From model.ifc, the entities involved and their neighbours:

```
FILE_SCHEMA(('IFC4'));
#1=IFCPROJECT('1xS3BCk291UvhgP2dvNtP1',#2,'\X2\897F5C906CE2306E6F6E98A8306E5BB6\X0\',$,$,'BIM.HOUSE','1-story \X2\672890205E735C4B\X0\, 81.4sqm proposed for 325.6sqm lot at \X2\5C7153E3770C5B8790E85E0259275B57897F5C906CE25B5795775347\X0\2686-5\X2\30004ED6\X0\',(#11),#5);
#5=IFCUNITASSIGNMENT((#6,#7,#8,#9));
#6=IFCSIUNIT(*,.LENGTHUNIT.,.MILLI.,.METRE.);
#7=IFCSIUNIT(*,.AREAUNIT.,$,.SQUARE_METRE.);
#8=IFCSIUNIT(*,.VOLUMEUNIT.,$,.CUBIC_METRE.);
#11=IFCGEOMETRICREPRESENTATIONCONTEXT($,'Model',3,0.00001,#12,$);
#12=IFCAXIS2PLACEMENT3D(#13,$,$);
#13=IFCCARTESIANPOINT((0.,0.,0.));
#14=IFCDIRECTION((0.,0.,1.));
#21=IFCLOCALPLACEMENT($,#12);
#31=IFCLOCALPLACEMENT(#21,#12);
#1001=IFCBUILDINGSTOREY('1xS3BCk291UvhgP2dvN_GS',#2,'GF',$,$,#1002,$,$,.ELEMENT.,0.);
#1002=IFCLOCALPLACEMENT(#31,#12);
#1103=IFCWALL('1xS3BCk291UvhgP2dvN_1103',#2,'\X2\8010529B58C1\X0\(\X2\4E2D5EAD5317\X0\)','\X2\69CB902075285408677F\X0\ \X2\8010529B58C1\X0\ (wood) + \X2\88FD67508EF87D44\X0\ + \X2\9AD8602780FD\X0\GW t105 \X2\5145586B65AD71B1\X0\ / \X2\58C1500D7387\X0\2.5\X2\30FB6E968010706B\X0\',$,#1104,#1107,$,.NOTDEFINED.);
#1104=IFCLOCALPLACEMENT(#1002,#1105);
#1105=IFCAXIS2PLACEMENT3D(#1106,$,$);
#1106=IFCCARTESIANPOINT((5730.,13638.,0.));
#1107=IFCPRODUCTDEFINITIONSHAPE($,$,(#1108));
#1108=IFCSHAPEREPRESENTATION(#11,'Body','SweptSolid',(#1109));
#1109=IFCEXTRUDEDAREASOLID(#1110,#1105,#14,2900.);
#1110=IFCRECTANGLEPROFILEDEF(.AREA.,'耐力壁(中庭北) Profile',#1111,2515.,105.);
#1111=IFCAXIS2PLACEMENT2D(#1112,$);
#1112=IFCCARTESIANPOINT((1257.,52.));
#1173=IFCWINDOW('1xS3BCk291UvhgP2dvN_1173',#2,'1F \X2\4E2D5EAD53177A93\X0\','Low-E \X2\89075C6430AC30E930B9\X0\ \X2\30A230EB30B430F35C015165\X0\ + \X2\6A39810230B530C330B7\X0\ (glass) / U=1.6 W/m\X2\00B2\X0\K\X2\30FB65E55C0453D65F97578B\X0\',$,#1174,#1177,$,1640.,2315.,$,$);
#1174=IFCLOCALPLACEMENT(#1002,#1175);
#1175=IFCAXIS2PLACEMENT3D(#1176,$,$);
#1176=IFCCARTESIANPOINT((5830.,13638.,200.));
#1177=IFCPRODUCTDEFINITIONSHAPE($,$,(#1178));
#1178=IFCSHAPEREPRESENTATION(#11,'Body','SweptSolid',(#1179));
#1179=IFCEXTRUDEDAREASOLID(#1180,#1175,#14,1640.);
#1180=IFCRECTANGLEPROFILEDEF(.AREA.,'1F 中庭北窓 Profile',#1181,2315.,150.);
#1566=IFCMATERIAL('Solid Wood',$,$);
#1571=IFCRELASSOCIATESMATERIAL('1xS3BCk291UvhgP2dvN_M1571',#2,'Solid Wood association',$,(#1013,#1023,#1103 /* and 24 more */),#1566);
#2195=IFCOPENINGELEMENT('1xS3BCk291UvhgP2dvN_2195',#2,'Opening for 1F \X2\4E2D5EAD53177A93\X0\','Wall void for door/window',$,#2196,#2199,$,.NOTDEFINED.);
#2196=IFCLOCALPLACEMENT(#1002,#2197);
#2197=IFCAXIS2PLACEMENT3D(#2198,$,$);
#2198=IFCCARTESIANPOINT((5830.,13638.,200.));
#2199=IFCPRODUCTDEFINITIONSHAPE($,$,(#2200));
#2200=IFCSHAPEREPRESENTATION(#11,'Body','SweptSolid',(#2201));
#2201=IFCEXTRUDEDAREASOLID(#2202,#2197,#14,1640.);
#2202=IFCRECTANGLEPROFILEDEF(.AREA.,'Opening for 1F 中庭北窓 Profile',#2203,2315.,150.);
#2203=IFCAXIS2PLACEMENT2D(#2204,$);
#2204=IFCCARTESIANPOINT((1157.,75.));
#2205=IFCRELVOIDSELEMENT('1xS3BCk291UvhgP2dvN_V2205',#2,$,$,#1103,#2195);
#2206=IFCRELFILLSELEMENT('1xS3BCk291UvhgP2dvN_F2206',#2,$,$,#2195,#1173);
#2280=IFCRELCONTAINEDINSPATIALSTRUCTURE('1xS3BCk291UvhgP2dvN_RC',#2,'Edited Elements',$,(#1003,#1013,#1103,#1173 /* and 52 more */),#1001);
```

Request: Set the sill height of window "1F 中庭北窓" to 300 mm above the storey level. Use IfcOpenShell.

```python
import numpy as np
import ifcopenshell
import ifcopenshell.api.geometry
import ifcopenshell.geom
import ifcopenshell.util.element
import ifcopenshell.util.placement
import ifcopenshell.util.shape
import ifcopenshell.util.unit

model = ifcopenshell.open("model.ifc")
unit_scale = ifcopenshell.util.unit.calculate_unit_scale(model)

window = model.by_id(1173)
opening = window.FillsVoids[0].RelatingOpeningElement
storey = ifcopenshell.util.element.get_container(window, ifc_class="IfcBuildingStorey")
level = ifcopenshell.util.placement.get_local_placement(storey.ObjectPlacement)[2, 3]

# The opening's origin need not be at the sill, so measure its lowest point.
shape = ifcopenshell.geom.create_shape(ifcopenshell.geom.settings(), opening)
bottom = ifcopenshell.util.shape.get_shape_bottom_elevation(shape, shape.geometry) / unit_scale
dz = level + 0.3 / unit_scale - bottom

shift = np.array([0.0, 0.0, dz])
# The window is not placed relative to its opening, so move both.
for product in (opening, window):
    matrix = ifcopenshell.util.placement.get_local_placement(product.ObjectPlacement)
    matrix[:3, 3] += shift
    ifcopenshell.api.geometry.edit_object_placement(model, product=product, matrix=matrix, is_si=False)

print(f"moved by {dz * unit_scale:+.3f} m")

model.write("model_edited.ifc")
```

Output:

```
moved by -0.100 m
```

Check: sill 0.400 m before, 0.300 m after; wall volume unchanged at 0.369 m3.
